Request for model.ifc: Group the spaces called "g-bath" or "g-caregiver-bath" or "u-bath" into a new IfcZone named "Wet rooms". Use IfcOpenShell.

First a look at what the model holds.

```python
import ifcopenshell

model = ifcopenshell.open("model.ifc")
print(model.schema)
seen = {}
for space in model.by_type("IfcSpace"):
    seen[space.LongName] = seen.get(space.LongName, 0) + 1
for name, count in sorted(seen.items(), key=str):
    print(count, "x", name)
print("zones:", [z.Name for z in model.by_type("IfcZone")][:20])
```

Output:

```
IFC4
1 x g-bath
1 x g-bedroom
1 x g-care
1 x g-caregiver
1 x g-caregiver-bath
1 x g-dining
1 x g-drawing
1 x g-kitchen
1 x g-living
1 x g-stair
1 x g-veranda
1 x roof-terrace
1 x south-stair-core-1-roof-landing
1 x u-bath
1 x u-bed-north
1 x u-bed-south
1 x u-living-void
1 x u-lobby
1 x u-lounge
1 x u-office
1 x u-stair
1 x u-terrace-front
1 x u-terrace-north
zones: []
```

```python
import ifcopenshell
import ifcopenshell.api.group
import ifcopenshell.api.root

model = ifcopenshell.open("model.ifc")

names = {"g-bath", "g-caregiver-bath", "u-bath"}
spaces = [s for s in model.by_type("IfcSpace") if s.LongName in names]

zone = ifcopenshell.api.root.create_entity(model, ifc_class="IfcZone", name="Wet rooms")
ifcopenshell.api.group.assign_group(model, products=spaces, group=zone)
print(len(spaces), "spaces in", zone.Name)

model.write("model-out.ifc")
```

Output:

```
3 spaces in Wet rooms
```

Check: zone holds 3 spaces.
